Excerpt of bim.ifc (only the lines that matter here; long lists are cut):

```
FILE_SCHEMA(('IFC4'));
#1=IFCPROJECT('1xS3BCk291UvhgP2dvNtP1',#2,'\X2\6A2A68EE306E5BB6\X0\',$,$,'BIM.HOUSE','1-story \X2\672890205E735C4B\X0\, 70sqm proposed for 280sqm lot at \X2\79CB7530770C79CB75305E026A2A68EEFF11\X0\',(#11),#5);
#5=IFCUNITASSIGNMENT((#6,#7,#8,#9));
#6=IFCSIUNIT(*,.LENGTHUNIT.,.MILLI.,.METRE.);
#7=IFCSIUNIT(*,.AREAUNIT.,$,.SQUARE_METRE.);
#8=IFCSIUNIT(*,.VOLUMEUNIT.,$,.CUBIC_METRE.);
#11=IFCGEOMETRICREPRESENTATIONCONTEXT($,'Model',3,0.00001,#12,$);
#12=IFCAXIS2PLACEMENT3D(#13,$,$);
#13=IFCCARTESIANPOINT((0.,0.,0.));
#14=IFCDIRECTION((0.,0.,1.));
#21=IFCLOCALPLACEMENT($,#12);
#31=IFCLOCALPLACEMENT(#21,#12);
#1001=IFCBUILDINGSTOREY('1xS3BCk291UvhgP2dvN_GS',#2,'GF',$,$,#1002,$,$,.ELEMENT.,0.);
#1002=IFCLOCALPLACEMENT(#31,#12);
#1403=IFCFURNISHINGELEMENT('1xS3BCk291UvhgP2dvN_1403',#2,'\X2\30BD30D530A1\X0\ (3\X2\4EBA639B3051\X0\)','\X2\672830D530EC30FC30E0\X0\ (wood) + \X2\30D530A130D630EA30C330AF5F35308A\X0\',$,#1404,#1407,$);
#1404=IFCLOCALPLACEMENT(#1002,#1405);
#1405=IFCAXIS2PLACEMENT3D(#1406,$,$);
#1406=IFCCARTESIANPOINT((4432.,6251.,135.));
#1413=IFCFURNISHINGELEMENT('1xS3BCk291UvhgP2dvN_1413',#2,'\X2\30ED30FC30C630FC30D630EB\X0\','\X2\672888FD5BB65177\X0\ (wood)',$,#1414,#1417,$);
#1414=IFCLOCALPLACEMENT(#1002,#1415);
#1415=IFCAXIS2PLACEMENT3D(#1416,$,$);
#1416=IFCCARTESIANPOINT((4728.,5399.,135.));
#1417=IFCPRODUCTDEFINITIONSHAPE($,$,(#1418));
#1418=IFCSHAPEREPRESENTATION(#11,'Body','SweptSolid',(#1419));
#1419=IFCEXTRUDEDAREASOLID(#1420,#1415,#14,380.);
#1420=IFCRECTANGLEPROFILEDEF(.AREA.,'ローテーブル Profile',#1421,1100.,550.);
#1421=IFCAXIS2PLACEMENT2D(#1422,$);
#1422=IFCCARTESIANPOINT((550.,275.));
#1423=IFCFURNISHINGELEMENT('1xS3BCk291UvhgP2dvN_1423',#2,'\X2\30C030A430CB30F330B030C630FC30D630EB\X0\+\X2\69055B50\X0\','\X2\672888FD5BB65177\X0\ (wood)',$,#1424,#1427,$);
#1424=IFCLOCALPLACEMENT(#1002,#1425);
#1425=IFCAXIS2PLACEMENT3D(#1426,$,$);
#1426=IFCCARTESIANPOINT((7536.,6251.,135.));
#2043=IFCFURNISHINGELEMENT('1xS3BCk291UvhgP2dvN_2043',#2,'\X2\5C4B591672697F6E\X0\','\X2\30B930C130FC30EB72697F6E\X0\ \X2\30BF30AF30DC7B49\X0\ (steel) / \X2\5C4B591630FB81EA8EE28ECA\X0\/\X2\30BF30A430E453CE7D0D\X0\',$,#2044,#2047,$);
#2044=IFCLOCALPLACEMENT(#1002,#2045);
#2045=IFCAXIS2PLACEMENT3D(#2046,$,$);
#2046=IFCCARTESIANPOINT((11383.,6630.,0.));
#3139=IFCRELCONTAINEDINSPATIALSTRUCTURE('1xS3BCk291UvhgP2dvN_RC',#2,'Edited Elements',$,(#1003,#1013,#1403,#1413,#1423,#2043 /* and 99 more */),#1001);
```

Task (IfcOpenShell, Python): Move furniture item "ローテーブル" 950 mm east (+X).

```python
import ifcopenshell
import ifcopenshell.api.geometry
import ifcopenshell.util.placement
import ifcopenshell.util.unit

model = ifcopenshell.open("bim.ifc")
unit_scale = ifcopenshell.util.unit.calculate_unit_scale(model)

item = model.by_guid("1xS3BCk291UvhgP2dvN_1413")
matrix = ifcopenshell.util.placement.get_local_placement(item.ObjectPlacement)
matrix[0, 3] += 0.95 / unit_scale
ifcopenshell.api.geometry.edit_object_placement(model, product=item, matrix=matrix, is_si=False)

print(ifcopenshell.util.placement.get_local_placement(item.ObjectPlacement).round(3) + 0.0)

model.write("bim_v2.ifc")
```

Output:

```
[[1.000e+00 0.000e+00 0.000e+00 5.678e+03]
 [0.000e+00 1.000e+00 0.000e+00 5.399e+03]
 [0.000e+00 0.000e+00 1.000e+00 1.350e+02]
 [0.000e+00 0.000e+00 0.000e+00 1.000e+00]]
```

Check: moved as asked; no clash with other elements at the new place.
